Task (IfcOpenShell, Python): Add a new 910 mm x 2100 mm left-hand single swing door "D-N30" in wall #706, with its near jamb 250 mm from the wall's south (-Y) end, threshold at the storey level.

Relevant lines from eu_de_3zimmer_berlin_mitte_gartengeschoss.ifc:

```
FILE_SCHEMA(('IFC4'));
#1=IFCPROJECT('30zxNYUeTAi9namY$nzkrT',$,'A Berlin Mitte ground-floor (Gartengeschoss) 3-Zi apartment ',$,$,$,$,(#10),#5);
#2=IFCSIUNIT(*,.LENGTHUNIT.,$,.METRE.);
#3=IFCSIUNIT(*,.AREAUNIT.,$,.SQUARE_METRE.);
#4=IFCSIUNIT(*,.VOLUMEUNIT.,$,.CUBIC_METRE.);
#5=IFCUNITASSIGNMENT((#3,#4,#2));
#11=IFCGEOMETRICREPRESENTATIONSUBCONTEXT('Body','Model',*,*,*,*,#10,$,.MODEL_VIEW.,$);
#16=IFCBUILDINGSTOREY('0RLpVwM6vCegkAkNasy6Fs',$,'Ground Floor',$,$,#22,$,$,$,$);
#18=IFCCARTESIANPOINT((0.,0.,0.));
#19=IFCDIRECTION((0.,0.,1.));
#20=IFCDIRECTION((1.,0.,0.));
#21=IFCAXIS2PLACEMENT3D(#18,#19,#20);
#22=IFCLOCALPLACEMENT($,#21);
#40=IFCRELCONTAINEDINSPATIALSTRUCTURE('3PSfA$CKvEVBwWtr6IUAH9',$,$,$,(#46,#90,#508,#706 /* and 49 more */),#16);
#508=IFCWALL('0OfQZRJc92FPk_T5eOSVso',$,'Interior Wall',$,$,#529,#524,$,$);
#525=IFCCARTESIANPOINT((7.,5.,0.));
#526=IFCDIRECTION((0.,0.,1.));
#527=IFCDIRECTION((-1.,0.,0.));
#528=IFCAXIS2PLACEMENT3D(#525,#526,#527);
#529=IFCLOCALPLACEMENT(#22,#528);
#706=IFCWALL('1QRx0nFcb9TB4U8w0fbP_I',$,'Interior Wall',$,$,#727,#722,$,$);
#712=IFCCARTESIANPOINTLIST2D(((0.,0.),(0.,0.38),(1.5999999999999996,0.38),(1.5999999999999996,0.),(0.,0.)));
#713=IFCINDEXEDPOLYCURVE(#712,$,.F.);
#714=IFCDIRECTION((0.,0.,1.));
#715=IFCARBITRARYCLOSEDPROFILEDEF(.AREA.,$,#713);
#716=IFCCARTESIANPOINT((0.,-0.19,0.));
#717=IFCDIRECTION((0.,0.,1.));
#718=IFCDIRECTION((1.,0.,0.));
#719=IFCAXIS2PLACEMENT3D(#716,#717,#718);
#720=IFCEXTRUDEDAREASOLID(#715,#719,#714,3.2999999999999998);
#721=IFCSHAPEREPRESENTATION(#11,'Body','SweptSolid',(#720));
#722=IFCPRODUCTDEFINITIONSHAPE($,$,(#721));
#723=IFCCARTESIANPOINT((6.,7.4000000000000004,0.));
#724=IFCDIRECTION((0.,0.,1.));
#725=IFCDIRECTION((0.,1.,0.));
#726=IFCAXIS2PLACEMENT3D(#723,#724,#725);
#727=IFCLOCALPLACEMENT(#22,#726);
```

```python
import numpy as np
import ifcopenshell
import ifcopenshell.api.feature
import ifcopenshell.api.geometry
import ifcopenshell.api.root
import ifcopenshell.api.spatial
import ifcopenshell.geom
import ifcopenshell.util.element
import ifcopenshell.util.placement
import ifcopenshell.util.representation
import ifcopenshell.util.shape
import ifcopenshell.util.unit

model = ifcopenshell.open("eu_de_3zimmer_berlin_mitte_gartengeschoss.ifc")
unit_scale = ifcopenshell.util.unit.calculate_unit_scale(model)
settings = ifcopenshell.geom.settings()


def volume(element):
    """Net volume in cubic metres, openings subtracted."""
    shape = ifcopenshell.geom.create_shape(settings, element)
    return ifcopenshell.util.shape.get_volume(shape.geometry)


wall = model.by_guid("1QRx0nFcb9TB4U8w0fbP_I")
storey = ifcopenshell.util.element.get_container(wall, ifc_class="IfcBuildingStorey")
context = ifcopenshell.util.representation.get_context(model, "Model", "Body", "MODEL_VIEW")
before = volume(wall)

width, height, from_end, sill = 0.91, 2.1, 0.25, 0.0  # metres

# The wall runs along its own X axis, and the end named is its -X end.
wall_shape = ifcopenshell.geom.create_shape(settings, wall)
x, y, z = ifcopenshell.util.shape.get_vertices(wall_shape.geometry).T
start = x.min() + from_end
face, thickness = float(y.min()), float(y.max() - y.min())
wall_matrix = ifcopenshell.util.placement.get_local_placement(wall.ObjectPlacement)
level = ifcopenshell.util.placement.get_local_placement(storey.ObjectPlacement)[2, 3]


def in_wall(x, y):
    """Placement at x, y metres in the wall's axes, at sill height."""
    matrix = wall_matrix.copy()
    matrix[:, 3] = wall_matrix @ np.array([x / unit_scale, y / unit_scale, 0.0, 1.0])
    matrix[2, 3] = level + sill / unit_scale
    return matrix


# Opening: a box that overshoots both wall faces by 50 mm.
opening = ifcopenshell.api.root.create_entity(model, ifc_class="IfcOpeningElement", predefined_type="OPENING")
box = ifcopenshell.api.geometry.add_wall_representation(
    model, context=context, length=width, height=height, thickness=thickness + 0.1
)
ifcopenshell.api.geometry.assign_representation(model, product=opening, representation=box)
ifcopenshell.api.geometry.edit_object_placement(model, product=opening, matrix=in_wall(start, face - 0.05), is_si=False)
ifcopenshell.api.feature.add_feature(model, feature=opening, element=wall)

door = ifcopenshell.api.root.create_entity(model, ifc_class="IfcDoor", name="D-N30", predefined_type="DOOR")
door.OverallWidth, door.OverallHeight = width / unit_scale, height / unit_scale
door.OperationType = "SINGLE_SWING_LEFT"
body = ifcopenshell.api.geometry.add_door_representation(
    model,
    context=context,
    overall_width=door.OverallWidth,
    overall_height=door.OverallHeight,
    operation_type="SINGLE_SWING_LEFT",
    lining_properties={"LiningDepth": thickness / unit_scale, "ThresholdDepth": thickness / unit_scale},
)
ifcopenshell.api.geometry.assign_representation(model, product=door, representation=body)
ifcopenshell.api.spatial.assign_container(model, products=[door], relating_structure=storey)
ifcopenshell.api.feature.add_filling(model, opening=opening, element=door)

# The lining spans the wall, so the door starts at the wall face.
ifcopenshell.api.geometry.edit_object_placement(model, product=door, matrix=in_wall(start, face), is_si=False)

after = volume(wall)

print(f"wall volume {before:.3f} -> {after:.3f} m3")

model.write("eu_de_3zimmer_berlin_mitte_gartengeschoss_edited.ifc")
```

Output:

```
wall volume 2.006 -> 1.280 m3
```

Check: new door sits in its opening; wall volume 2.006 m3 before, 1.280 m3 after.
